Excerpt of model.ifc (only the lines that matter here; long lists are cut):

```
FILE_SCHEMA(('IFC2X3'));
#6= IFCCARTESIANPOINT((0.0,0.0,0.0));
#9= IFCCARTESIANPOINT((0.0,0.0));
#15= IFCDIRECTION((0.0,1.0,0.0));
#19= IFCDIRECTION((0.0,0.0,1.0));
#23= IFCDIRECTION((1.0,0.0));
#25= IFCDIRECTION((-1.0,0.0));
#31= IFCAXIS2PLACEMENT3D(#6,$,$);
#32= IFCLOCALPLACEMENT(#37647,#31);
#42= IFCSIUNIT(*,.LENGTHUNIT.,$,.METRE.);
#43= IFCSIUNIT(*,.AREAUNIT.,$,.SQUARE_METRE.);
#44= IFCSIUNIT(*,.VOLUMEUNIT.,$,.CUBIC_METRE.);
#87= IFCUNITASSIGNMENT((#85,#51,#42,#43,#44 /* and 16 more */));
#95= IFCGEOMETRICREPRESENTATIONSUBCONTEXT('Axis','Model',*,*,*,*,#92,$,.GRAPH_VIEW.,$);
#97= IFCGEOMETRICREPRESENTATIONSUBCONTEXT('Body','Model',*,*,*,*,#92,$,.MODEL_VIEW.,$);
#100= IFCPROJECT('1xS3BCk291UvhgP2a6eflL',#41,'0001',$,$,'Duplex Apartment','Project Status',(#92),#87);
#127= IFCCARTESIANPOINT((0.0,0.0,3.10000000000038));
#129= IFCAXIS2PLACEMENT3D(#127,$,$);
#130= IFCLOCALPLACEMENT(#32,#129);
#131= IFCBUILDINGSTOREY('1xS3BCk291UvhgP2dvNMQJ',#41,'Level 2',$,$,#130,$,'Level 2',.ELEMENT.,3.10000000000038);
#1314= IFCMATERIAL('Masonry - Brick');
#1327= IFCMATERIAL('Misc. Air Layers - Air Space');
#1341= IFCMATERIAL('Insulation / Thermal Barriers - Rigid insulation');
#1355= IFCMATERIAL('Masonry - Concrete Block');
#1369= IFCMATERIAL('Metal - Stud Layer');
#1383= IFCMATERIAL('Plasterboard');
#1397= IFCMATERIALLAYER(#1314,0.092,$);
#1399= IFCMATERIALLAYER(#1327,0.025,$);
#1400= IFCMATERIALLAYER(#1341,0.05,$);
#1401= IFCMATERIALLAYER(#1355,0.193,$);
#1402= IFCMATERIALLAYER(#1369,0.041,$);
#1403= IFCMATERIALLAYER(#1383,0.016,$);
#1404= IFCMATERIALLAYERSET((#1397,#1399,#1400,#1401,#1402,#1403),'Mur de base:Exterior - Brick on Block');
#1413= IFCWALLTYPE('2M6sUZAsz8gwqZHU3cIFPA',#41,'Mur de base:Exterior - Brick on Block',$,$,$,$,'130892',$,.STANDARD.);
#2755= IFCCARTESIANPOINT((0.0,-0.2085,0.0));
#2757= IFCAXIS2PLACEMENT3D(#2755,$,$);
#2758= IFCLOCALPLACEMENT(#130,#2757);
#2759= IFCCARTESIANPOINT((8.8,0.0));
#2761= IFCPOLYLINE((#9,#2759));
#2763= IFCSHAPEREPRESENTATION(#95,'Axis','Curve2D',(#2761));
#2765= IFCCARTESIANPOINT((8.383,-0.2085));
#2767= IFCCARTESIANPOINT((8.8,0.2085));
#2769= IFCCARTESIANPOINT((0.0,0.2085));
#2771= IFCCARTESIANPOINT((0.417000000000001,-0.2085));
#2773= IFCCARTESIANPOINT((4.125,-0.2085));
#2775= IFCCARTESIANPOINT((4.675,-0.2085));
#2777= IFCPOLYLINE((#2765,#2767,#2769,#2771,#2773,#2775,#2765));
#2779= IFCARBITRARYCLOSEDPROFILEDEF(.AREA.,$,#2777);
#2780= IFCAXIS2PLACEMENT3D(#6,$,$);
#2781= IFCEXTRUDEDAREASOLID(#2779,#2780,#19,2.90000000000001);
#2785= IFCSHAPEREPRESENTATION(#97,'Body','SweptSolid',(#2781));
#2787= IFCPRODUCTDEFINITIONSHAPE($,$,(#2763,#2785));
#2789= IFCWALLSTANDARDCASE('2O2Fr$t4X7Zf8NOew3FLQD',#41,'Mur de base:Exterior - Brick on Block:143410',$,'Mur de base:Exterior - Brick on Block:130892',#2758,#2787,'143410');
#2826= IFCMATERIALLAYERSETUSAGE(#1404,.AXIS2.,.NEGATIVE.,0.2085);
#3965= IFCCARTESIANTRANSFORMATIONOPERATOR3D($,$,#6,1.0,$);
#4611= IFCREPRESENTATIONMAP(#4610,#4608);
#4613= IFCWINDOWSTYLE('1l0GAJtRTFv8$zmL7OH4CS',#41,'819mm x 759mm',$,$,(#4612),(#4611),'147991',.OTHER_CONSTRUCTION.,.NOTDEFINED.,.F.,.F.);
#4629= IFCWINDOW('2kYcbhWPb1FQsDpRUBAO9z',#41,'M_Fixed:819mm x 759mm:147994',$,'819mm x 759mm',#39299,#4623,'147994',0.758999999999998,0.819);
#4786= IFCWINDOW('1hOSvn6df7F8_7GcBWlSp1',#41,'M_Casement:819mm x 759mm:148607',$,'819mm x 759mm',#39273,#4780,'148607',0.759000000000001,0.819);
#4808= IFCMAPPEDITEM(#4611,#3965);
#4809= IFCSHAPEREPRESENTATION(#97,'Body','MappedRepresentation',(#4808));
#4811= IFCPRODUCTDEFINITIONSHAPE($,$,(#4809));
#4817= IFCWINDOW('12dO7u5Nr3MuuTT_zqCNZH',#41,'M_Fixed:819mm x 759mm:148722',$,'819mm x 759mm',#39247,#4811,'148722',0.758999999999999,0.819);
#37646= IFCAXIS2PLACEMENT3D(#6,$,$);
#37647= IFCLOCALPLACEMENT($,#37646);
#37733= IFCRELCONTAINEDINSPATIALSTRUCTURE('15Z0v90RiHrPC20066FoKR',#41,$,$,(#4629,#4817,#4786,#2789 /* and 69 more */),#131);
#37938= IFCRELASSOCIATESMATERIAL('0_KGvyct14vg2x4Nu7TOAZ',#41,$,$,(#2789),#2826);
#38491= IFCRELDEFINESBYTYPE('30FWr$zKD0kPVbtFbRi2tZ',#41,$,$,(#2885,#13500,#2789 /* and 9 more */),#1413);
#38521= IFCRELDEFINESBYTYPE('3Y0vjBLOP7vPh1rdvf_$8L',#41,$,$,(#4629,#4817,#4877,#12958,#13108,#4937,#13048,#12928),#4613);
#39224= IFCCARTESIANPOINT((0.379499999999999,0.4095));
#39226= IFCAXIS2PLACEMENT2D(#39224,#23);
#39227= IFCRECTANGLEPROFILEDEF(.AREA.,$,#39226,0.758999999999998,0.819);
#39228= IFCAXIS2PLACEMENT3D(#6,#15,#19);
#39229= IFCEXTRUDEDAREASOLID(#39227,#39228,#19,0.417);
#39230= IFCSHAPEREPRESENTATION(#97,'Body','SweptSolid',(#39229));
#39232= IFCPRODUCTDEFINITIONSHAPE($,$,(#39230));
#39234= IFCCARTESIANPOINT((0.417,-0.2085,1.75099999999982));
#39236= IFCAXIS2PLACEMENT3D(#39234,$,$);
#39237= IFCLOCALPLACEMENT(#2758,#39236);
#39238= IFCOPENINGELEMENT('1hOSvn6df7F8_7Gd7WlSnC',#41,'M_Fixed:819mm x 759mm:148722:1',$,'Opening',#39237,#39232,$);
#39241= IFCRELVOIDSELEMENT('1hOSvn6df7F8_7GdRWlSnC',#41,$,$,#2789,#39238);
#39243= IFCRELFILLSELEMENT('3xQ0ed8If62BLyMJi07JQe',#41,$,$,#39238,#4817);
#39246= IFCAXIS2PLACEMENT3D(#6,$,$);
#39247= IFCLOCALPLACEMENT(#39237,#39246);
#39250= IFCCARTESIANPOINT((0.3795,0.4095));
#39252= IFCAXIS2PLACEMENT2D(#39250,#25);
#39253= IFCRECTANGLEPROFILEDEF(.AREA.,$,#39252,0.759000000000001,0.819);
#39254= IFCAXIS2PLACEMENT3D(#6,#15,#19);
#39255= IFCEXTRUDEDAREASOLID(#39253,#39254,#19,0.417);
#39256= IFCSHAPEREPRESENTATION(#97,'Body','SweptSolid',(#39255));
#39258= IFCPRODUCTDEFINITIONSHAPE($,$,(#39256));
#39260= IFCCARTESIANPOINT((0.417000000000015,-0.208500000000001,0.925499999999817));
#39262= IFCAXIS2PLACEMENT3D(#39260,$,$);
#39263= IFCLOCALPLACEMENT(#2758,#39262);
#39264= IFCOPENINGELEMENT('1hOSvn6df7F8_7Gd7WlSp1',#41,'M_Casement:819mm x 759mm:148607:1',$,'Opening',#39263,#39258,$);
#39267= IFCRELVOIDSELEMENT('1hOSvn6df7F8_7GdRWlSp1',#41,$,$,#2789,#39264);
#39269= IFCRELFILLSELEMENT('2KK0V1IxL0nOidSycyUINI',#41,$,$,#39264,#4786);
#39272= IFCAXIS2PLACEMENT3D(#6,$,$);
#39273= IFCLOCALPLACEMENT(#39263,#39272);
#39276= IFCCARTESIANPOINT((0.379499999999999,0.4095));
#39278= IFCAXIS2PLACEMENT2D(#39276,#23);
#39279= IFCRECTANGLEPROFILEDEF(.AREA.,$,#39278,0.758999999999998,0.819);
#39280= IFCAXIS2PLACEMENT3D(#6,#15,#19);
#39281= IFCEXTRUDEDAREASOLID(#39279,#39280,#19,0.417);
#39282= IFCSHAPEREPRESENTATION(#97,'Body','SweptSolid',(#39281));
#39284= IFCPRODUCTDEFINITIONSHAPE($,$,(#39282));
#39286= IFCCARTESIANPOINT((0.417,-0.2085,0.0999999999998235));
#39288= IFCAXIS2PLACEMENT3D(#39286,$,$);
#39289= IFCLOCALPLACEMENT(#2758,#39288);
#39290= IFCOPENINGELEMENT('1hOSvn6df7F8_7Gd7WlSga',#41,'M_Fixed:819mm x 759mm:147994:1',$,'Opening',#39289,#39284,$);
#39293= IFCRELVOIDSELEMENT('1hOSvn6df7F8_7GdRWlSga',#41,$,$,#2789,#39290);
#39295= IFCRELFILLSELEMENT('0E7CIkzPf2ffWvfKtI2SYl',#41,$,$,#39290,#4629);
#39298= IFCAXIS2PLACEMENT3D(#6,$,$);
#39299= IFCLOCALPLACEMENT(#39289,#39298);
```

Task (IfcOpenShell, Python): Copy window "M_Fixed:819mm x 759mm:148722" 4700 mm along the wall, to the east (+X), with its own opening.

```python
import ifcopenshell
import ifcopenshell.api.feature
import ifcopenshell.api.geometry
import ifcopenshell.api.root
import ifcopenshell.geom
import ifcopenshell.util.element
import ifcopenshell.util.placement
import ifcopenshell.util.shape
import ifcopenshell.util.unit

model = ifcopenshell.open("model.ifc")
unit_scale = ifcopenshell.util.unit.calculate_unit_scale(model)
settings = ifcopenshell.geom.settings()


def volume(element):
    """Net volume in cubic metres, openings subtracted."""
    shape = ifcopenshell.geom.create_shape(settings, element)
    return ifcopenshell.util.shape.get_volume(shape.geometry)


def reuse_history(source, copy):
    """copy_class also copies each property set's owner history, people and application; keep the originals."""
    for rel in copy.IsDefinedBy:
        if rel.is_a("IfcRelDefinesByProperties") and (history := rel.RelatingPropertyDefinition.OwnerHistory):
            rel.RelatingPropertyDefinition.OwnerHistory = source.OwnerHistory
            ifcopenshell.util.element.remove_deep2(model, history)


window = model.by_guid("12dO7u5Nr3MuuTT_zqCNZH")
opening = window.FillsVoids[0].RelatingOpeningElement
wall = opening.VoidsElements[0].RelatingBuildingElement
before = volume(wall)
shift = ifcopenshell.util.placement.get_local_placement(wall.ObjectPlacement)[:3, 0] * 4.7 / unit_scale

# copy_class copies the void relationship, type, container and properties, but no geometry.
new_opening = ifcopenshell.api.root.copy_class(model, product=opening)
new_opening.Representation = ifcopenshell.util.element.copy_deep(
    model, opening.Representation, exclude=["IfcGeometricRepresentationContext", "IfcRepresentationMap"]
)
new_opening.Name = "M_Fixed:819mm x 759mm"
new_window = ifcopenshell.api.root.copy_class(model, product=window)
new_window.Representation = ifcopenshell.util.element.copy_deep(
    model, window.Representation, exclude=["IfcGeometricRepresentationContext", "IfcRepresentationMap"]
)
new_window.Name = "M_Fixed:819mm x 759mm"
new_window.Tag = None
reuse_history(window, new_window)
fills = ifcopenshell.api.feature.add_filling(model, opening=new_opening, element=new_window)
fills.OwnerHistory = new_window.OwnerHistory  # required in IFC2X3

for old, new in ((opening, new_opening), (window, new_window)):
    matrix = ifcopenshell.util.placement.get_local_placement(old.ObjectPlacement)
    matrix[:3, 3] += shift
    ifcopenshell.api.geometry.edit_object_placement(model, product=new, matrix=matrix, is_si=False)

after = volume(wall)

print(f"wall volume {before:.3f} -> {after:.3f} m3")

model.write("model-out.ifc")
```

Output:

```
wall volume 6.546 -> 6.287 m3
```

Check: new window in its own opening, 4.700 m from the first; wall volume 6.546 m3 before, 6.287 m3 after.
